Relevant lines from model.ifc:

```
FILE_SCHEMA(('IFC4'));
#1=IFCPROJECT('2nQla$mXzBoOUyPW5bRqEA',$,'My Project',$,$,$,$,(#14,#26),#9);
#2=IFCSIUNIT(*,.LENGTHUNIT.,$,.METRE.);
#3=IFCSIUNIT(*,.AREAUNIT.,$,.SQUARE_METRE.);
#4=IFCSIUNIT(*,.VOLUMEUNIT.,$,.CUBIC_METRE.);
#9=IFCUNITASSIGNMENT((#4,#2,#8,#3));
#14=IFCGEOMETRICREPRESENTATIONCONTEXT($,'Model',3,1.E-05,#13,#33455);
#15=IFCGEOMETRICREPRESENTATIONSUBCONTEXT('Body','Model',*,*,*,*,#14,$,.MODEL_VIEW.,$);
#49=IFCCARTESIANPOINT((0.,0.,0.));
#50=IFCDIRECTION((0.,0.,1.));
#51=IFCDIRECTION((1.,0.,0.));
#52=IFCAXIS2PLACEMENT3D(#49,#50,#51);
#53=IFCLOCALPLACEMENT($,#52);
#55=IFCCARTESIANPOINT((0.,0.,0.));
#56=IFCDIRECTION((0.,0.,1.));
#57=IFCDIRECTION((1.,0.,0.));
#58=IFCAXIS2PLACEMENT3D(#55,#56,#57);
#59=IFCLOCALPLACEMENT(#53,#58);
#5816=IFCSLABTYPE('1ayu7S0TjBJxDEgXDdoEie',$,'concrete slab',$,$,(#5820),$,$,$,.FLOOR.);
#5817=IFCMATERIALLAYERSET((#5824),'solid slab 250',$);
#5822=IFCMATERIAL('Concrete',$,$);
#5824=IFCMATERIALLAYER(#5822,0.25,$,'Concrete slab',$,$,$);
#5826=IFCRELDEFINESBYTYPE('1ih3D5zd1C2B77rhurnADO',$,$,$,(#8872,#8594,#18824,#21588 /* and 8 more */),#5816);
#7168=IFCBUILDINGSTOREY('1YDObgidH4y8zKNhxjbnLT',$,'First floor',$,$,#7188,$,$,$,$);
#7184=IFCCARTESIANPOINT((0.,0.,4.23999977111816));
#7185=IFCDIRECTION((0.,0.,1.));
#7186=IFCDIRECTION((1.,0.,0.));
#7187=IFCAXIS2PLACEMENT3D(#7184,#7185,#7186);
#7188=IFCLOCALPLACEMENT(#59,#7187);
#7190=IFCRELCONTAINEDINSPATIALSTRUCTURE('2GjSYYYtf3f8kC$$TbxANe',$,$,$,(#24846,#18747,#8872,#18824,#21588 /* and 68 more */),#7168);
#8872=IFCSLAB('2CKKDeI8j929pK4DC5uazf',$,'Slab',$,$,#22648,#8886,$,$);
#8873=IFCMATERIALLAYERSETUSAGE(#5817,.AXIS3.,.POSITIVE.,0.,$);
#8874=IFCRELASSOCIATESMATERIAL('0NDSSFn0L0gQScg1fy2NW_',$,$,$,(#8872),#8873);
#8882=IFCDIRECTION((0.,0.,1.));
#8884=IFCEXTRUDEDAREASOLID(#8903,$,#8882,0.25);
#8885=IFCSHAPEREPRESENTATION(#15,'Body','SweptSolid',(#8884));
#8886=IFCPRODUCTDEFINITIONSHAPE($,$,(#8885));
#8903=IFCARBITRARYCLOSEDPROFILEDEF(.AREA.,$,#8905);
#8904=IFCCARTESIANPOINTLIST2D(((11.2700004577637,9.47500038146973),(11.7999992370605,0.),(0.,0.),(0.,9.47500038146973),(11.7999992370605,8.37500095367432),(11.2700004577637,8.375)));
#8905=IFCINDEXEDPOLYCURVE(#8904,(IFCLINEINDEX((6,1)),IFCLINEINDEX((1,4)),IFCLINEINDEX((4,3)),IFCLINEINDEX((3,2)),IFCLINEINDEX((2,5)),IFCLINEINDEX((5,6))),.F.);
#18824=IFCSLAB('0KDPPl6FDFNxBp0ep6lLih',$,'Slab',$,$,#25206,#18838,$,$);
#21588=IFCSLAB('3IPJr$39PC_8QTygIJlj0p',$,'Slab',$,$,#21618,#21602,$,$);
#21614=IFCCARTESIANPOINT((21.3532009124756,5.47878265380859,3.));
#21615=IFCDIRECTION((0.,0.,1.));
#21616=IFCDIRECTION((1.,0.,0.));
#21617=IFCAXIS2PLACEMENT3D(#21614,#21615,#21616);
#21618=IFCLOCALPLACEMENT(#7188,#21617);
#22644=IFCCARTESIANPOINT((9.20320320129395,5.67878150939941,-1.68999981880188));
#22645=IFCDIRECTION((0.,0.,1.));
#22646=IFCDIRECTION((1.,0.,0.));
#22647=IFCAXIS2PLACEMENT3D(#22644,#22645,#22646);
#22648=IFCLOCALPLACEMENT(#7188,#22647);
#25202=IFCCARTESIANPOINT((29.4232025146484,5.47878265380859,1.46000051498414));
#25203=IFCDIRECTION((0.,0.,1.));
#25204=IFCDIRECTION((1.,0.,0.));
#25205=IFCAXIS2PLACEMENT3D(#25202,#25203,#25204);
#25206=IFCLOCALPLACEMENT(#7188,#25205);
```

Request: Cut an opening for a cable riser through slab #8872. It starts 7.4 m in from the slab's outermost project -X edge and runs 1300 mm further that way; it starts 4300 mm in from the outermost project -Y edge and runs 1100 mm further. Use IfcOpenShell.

```python
import numpy as np
import ifcopenshell
import ifcopenshell.api.feature
import ifcopenshell.api.geometry
import ifcopenshell.api.root
import ifcopenshell.geom
import ifcopenshell.util.placement
import ifcopenshell.util.representation
import ifcopenshell.util.shape
import ifcopenshell.util.unit

model = ifcopenshell.open("model.ifc")
unit_scale = ifcopenshell.util.unit.calculate_unit_scale(model)
settings = ifcopenshell.geom.settings()


def volume(element):
    """Net volume in cubic metres, openings subtracted."""
    shape = ifcopenshell.geom.create_shape(settings, element)
    return ifcopenshell.util.shape.get_volume(shape.geometry)


slab = model.by_guid("2CKKDeI8j929pK4DC5uazf")
before = volume(slab)

# Extent in the slab's own axes, in metres. The edges named are its -X and -Y sides.
slab_shape = ifcopenshell.geom.create_shape(settings, slab)
vertices = ifcopenshell.util.shape.get_vertices(slab_shape.geometry)
x_min, y_min, bottom = vertices.min(axis=0)
top = vertices[:, 2].max()

opening = ifcopenshell.api.root.create_entity(model, ifc_class="IfcOpeningElement", name="Cable riser opening", predefined_type="OPENING")
context = ifcopenshell.util.representation.get_context(model, "Model", "Body", "MODEL_VIEW")
width, depth = 1.3, 1.1
outline = [(0.0, 0.0), (width, 0.0), (width, depth), (0.0, depth), (0.0, 0.0)]
# Overshoot both faces by 50 mm so the cut is clean.
shape = ifcopenshell.api.geometry.add_slab_representation(
    model, context=context, depth=top - bottom + 0.1, polyline=outline
)
ifcopenshell.api.geometry.assign_representation(model, product=opening, representation=shape)

matrix = ifcopenshell.util.placement.get_local_placement(slab.ObjectPlacement)
matrix[:, 3] = matrix @ np.append(np.array([x_min + 7.4, y_min + 4.3, bottom - 0.05]) / unit_scale, 1.0)
ifcopenshell.api.geometry.edit_object_placement(model, product=opening, matrix=matrix, is_si=False)
ifcopenshell.api.feature.add_feature(model, feature=opening, element=slab)

after = volume(slab)

print(f"slab volume {before:.3f} -> {after:.3f} m3")

model.write("model_rev.ifc")
```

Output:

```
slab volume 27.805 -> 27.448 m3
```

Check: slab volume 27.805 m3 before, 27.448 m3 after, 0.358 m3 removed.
